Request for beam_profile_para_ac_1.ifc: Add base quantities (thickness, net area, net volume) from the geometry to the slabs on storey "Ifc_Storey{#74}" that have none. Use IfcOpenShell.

First a look at what the model holds.

```python
import ifcopenshell
import ifcopenshell.util.element
import ifcopenshell.util.unit

model = ifcopenshell.open("beam_profile_para_ac_1.ifc")
print(model.schema)
for unit_type in ("LENGTHUNIT", "AREAUNIT", "VOLUMEUNIT"):
    print(unit_type, ifcopenshell.util.unit.calculate_unit_scale(model, unit_type))
storey = next(s for s in model.by_type("IfcBuildingStorey") if s.Name == "Ifc_Storey{#74}")
slabs = [e for e in ifcopenshell.util.element.get_decomposition(storey) if e.is_a("IfcSlab")]
for e in sorted(slabs, key=lambda e: e.id()):
    print(e.id(), e.is_a(), e.Name, list(ifcopenshell.util.element.get_psets(e, qtos_only=True)), sep=" | ")
```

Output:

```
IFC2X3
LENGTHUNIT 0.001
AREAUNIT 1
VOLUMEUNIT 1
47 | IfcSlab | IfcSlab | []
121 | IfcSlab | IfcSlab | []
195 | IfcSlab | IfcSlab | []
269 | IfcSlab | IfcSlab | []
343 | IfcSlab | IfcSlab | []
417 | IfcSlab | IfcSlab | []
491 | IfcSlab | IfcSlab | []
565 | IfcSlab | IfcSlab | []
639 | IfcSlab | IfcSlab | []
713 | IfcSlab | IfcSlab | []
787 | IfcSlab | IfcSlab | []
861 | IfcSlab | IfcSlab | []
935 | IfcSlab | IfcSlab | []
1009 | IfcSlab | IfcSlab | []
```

```python
import ifcopenshell
import ifcopenshell.api.pset
import ifcopenshell.geom
import ifcopenshell.util.element
import ifcopenshell.util.shape
import ifcopenshell.util.unit

model = ifcopenshell.open("beam_profile_para_ac_1.ifc")
unit_scale = ifcopenshell.util.unit.calculate_unit_scale(model)
area_scale = ifcopenshell.util.unit.calculate_unit_scale(model, "AREAUNIT")
volume_scale = ifcopenshell.util.unit.calculate_unit_scale(model, "VOLUMEUNIT")
settings = ifcopenshell.geom.settings()

storey = next(s for s in model.by_type("IfcBuildingStorey") if s.Name == "Ifc_Storey{#74}")
slabs = [e for e in ifcopenshell.util.element.get_decomposition(storey) if e.is_a("IfcSlab")]

for e in sorted(slabs, key=lambda e: e.id()):
    if ifcopenshell.util.element.get_psets(e, qtos_only=True, should_inherit=False):
        continue
    # Geometry comes back in metres, in the element's own axes.
    shape = ifcopenshell.geom.create_shape(settings, e)
    values = {
        "Width": ifcopenshell.util.shape.get_z(shape.geometry) / unit_scale,
        "NetArea": ifcopenshell.util.shape.get_footprint_area(shape.geometry) / area_scale,
        "NetVolume": ifcopenshell.util.shape.get_volume(shape.geometry) / volume_scale,
    }
    qto = ifcopenshell.api.pset.add_qto(model, product=e, name="BaseQuantities")
    ifcopenshell.api.pset.edit_qto(model, qto=qto, properties=values)
    print(e.id(), {k: round(v, 3) for k, v in values.items()})

model.write("beam_profile_para_ac_1_v2.ifc")
```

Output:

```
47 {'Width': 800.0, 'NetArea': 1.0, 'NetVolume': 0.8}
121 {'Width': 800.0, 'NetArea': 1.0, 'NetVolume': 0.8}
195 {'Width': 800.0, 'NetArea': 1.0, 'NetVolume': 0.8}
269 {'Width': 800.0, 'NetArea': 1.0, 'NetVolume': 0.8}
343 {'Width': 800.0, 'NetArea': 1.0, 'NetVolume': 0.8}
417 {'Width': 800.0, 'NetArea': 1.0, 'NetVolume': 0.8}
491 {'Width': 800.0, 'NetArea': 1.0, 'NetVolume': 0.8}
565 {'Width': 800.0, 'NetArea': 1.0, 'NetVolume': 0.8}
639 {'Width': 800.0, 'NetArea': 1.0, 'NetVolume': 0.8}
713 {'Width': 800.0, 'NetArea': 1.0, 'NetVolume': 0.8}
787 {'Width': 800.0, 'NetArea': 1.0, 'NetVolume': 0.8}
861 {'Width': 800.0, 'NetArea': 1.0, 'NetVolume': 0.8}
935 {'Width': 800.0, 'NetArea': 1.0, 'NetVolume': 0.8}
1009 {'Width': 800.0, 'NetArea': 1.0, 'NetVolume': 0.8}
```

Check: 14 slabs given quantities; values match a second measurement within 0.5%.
